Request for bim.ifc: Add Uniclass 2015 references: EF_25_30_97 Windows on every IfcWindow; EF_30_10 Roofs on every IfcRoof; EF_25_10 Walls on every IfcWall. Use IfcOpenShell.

First a look at what the model holds.

```python
import ifcopenshell

model = ifcopenshell.open("bim.ifc")
print(model.schema)
print("classifications:", [c.Name for c in model.by_type("IfcClassification")])
for ifc_class in ("IfcDoor", "IfcRoof", "IfcStair", "IfcWall", "IfcWindow"):
    print(ifc_class, len(model.by_type(ifc_class)))
```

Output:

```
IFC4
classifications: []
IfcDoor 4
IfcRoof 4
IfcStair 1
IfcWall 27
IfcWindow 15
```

```python
import ifcopenshell
import ifcopenshell.api.classification

model = ifcopenshell.open("bim.ifc")

system = ifcopenshell.api.classification.add_classification(model, classification="Uniclass 2015")

codes = {
    "IfcWindow": ("EF_25_30_97", "Windows"),
    "IfcRoof": ("EF_30_10", "Roofs"),
    "IfcWall": ("EF_25_10", "Walls"),
}
for ifc_class, (code, name) in codes.items():
    products = model.by_type(ifc_class)
    ifcopenshell.api.classification.add_reference(
        model, products=products, classification=system, identification=code, name=name
    )
    print(code, len(products))

model.write("bim_edited.ifc")
```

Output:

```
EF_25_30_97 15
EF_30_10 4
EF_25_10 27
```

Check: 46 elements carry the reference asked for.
